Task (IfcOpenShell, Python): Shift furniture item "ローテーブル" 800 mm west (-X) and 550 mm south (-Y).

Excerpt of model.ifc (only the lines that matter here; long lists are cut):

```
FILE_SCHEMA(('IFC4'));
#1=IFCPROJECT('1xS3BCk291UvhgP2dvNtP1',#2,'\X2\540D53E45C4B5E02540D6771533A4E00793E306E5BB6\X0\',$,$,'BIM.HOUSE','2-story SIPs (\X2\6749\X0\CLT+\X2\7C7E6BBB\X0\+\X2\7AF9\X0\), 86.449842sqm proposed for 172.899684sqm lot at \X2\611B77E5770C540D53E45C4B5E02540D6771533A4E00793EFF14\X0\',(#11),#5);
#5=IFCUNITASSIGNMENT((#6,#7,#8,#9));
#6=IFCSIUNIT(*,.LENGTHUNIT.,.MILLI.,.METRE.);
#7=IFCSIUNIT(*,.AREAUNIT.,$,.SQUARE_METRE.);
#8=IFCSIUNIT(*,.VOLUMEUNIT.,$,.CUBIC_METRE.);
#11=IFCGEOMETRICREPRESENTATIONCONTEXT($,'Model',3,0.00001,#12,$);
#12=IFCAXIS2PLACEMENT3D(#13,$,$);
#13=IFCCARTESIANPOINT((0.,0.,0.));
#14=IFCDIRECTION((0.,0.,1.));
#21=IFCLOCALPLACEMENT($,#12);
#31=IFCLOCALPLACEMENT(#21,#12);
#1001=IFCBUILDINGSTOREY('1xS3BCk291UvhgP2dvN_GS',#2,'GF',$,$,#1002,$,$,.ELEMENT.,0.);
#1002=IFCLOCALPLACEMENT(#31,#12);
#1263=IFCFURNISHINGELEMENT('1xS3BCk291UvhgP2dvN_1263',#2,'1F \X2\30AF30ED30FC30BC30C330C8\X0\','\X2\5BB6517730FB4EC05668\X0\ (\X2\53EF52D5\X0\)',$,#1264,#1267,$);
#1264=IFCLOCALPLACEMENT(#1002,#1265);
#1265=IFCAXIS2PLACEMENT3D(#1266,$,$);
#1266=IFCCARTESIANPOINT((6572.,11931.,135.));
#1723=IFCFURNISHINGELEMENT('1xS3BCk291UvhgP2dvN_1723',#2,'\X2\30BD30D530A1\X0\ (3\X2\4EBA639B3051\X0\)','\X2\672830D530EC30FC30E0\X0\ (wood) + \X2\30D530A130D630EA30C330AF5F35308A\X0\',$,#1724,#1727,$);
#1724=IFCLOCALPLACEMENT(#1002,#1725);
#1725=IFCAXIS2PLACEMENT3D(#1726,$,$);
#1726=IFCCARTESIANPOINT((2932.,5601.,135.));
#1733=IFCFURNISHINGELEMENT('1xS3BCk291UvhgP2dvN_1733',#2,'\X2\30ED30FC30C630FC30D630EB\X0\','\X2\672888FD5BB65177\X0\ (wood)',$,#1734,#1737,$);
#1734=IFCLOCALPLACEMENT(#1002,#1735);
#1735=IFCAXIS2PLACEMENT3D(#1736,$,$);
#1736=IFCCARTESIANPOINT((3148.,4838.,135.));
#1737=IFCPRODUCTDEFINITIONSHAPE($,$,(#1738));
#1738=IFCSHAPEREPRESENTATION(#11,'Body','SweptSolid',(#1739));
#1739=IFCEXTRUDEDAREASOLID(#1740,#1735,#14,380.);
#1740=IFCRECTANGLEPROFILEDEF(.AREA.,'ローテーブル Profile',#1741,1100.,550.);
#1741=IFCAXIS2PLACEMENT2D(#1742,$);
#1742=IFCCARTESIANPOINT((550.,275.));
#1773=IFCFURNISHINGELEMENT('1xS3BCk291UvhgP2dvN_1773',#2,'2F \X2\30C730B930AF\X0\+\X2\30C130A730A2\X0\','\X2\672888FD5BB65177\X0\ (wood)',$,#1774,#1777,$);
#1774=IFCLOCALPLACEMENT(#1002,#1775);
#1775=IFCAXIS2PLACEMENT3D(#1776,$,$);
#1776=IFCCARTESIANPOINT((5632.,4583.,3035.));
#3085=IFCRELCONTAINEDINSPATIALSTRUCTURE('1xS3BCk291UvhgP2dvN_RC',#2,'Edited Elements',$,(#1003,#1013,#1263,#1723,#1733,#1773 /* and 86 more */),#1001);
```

```python
import ifcopenshell
import ifcopenshell.api.geometry
import ifcopenshell.util.placement
import ifcopenshell.util.unit

model = ifcopenshell.open("model.ifc")
unit_scale = ifcopenshell.util.unit.calculate_unit_scale(model)

item = model.by_id(1733)
matrix = ifcopenshell.util.placement.get_local_placement(item.ObjectPlacement)
matrix[0, 3] -= 0.8 / unit_scale
matrix[1, 3] -= 0.55 / unit_scale
ifcopenshell.api.geometry.edit_object_placement(model, product=item, matrix=matrix, is_si=False)

print(ifcopenshell.util.placement.get_local_placement(item.ObjectPlacement).round(3) + 0.0)

model.write("model_v2.ifc")
```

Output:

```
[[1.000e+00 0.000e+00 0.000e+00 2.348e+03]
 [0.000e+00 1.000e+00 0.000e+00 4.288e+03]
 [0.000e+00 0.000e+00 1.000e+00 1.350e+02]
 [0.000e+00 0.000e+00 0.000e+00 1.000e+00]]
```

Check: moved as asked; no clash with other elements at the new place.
